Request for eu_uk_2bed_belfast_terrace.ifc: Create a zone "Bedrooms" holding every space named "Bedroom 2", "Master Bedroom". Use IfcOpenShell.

First a look at what the model holds.

```python
import ifcopenshell

model = ifcopenshell.open("eu_uk_2bed_belfast_terrace.ifc")
print(model.schema)
seen = {}
for space in model.by_type("IfcSpace"):
    seen[space.LongName] = seen.get(space.LongName, 0) + 1
for name, count in sorted(seen.items(), key=str):
    print(count, "x", name)
print("zones:", [z.Name for z in model.by_type("IfcZone")][:20])
```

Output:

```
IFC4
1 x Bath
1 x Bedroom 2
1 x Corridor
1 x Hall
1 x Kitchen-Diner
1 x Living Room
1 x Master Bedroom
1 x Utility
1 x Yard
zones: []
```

```python
import ifcopenshell
import ifcopenshell.api.group
import ifcopenshell.api.root

model = ifcopenshell.open("eu_uk_2bed_belfast_terrace.ifc")

names = {"Bedroom 2", "Master Bedroom"}
spaces = [s for s in model.by_type("IfcSpace") if s.LongName in names]

zone = ifcopenshell.api.root.create_entity(model, ifc_class="IfcZone", name="Bedrooms")
ifcopenshell.api.group.assign_group(model, products=spaces, group=zone)
print(len(spaces), "spaces in", zone.Name)

model.write("eu_uk_2bed_belfast_terrace_rev.ifc")
```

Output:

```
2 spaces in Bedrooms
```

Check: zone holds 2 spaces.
